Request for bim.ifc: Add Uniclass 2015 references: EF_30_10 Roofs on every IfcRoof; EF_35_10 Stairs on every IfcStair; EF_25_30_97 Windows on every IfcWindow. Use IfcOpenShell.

First a look at what the model holds.

```python
import ifcopenshell

model = ifcopenshell.open("bim.ifc")
print(model.schema)
print("classifications:", [c.Name for c in model.by_type("IfcClassification")])
for ifc_class in ("IfcDoor", "IfcRoof", "IfcStair", "IfcWall", "IfcWindow"):
    print(ifc_class, len(model.by_type(ifc_class)))
```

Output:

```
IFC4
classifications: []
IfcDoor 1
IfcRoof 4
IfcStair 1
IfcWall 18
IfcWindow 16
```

```python
import ifcopenshell
import ifcopenshell.api.classification

model = ifcopenshell.open("bim.ifc")

system = ifcopenshell.api.classification.add_classification(model, classification="Uniclass 2015")

codes = {
    "IfcRoof": ("EF_30_10", "Roofs"),
    "IfcStair": ("EF_35_10", "Stairs"),
    "IfcWindow": ("EF_25_30_97", "Windows"),
}
for ifc_class, (code, name) in codes.items():
    products = model.by_type(ifc_class)
    ifcopenshell.api.classification.add_reference(
        model, products=products, classification=system, identification=code, name=name
    )
    print(code, len(products))

model.write("bim_edited.ifc")
```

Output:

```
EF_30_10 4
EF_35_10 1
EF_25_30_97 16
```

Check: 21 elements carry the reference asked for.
